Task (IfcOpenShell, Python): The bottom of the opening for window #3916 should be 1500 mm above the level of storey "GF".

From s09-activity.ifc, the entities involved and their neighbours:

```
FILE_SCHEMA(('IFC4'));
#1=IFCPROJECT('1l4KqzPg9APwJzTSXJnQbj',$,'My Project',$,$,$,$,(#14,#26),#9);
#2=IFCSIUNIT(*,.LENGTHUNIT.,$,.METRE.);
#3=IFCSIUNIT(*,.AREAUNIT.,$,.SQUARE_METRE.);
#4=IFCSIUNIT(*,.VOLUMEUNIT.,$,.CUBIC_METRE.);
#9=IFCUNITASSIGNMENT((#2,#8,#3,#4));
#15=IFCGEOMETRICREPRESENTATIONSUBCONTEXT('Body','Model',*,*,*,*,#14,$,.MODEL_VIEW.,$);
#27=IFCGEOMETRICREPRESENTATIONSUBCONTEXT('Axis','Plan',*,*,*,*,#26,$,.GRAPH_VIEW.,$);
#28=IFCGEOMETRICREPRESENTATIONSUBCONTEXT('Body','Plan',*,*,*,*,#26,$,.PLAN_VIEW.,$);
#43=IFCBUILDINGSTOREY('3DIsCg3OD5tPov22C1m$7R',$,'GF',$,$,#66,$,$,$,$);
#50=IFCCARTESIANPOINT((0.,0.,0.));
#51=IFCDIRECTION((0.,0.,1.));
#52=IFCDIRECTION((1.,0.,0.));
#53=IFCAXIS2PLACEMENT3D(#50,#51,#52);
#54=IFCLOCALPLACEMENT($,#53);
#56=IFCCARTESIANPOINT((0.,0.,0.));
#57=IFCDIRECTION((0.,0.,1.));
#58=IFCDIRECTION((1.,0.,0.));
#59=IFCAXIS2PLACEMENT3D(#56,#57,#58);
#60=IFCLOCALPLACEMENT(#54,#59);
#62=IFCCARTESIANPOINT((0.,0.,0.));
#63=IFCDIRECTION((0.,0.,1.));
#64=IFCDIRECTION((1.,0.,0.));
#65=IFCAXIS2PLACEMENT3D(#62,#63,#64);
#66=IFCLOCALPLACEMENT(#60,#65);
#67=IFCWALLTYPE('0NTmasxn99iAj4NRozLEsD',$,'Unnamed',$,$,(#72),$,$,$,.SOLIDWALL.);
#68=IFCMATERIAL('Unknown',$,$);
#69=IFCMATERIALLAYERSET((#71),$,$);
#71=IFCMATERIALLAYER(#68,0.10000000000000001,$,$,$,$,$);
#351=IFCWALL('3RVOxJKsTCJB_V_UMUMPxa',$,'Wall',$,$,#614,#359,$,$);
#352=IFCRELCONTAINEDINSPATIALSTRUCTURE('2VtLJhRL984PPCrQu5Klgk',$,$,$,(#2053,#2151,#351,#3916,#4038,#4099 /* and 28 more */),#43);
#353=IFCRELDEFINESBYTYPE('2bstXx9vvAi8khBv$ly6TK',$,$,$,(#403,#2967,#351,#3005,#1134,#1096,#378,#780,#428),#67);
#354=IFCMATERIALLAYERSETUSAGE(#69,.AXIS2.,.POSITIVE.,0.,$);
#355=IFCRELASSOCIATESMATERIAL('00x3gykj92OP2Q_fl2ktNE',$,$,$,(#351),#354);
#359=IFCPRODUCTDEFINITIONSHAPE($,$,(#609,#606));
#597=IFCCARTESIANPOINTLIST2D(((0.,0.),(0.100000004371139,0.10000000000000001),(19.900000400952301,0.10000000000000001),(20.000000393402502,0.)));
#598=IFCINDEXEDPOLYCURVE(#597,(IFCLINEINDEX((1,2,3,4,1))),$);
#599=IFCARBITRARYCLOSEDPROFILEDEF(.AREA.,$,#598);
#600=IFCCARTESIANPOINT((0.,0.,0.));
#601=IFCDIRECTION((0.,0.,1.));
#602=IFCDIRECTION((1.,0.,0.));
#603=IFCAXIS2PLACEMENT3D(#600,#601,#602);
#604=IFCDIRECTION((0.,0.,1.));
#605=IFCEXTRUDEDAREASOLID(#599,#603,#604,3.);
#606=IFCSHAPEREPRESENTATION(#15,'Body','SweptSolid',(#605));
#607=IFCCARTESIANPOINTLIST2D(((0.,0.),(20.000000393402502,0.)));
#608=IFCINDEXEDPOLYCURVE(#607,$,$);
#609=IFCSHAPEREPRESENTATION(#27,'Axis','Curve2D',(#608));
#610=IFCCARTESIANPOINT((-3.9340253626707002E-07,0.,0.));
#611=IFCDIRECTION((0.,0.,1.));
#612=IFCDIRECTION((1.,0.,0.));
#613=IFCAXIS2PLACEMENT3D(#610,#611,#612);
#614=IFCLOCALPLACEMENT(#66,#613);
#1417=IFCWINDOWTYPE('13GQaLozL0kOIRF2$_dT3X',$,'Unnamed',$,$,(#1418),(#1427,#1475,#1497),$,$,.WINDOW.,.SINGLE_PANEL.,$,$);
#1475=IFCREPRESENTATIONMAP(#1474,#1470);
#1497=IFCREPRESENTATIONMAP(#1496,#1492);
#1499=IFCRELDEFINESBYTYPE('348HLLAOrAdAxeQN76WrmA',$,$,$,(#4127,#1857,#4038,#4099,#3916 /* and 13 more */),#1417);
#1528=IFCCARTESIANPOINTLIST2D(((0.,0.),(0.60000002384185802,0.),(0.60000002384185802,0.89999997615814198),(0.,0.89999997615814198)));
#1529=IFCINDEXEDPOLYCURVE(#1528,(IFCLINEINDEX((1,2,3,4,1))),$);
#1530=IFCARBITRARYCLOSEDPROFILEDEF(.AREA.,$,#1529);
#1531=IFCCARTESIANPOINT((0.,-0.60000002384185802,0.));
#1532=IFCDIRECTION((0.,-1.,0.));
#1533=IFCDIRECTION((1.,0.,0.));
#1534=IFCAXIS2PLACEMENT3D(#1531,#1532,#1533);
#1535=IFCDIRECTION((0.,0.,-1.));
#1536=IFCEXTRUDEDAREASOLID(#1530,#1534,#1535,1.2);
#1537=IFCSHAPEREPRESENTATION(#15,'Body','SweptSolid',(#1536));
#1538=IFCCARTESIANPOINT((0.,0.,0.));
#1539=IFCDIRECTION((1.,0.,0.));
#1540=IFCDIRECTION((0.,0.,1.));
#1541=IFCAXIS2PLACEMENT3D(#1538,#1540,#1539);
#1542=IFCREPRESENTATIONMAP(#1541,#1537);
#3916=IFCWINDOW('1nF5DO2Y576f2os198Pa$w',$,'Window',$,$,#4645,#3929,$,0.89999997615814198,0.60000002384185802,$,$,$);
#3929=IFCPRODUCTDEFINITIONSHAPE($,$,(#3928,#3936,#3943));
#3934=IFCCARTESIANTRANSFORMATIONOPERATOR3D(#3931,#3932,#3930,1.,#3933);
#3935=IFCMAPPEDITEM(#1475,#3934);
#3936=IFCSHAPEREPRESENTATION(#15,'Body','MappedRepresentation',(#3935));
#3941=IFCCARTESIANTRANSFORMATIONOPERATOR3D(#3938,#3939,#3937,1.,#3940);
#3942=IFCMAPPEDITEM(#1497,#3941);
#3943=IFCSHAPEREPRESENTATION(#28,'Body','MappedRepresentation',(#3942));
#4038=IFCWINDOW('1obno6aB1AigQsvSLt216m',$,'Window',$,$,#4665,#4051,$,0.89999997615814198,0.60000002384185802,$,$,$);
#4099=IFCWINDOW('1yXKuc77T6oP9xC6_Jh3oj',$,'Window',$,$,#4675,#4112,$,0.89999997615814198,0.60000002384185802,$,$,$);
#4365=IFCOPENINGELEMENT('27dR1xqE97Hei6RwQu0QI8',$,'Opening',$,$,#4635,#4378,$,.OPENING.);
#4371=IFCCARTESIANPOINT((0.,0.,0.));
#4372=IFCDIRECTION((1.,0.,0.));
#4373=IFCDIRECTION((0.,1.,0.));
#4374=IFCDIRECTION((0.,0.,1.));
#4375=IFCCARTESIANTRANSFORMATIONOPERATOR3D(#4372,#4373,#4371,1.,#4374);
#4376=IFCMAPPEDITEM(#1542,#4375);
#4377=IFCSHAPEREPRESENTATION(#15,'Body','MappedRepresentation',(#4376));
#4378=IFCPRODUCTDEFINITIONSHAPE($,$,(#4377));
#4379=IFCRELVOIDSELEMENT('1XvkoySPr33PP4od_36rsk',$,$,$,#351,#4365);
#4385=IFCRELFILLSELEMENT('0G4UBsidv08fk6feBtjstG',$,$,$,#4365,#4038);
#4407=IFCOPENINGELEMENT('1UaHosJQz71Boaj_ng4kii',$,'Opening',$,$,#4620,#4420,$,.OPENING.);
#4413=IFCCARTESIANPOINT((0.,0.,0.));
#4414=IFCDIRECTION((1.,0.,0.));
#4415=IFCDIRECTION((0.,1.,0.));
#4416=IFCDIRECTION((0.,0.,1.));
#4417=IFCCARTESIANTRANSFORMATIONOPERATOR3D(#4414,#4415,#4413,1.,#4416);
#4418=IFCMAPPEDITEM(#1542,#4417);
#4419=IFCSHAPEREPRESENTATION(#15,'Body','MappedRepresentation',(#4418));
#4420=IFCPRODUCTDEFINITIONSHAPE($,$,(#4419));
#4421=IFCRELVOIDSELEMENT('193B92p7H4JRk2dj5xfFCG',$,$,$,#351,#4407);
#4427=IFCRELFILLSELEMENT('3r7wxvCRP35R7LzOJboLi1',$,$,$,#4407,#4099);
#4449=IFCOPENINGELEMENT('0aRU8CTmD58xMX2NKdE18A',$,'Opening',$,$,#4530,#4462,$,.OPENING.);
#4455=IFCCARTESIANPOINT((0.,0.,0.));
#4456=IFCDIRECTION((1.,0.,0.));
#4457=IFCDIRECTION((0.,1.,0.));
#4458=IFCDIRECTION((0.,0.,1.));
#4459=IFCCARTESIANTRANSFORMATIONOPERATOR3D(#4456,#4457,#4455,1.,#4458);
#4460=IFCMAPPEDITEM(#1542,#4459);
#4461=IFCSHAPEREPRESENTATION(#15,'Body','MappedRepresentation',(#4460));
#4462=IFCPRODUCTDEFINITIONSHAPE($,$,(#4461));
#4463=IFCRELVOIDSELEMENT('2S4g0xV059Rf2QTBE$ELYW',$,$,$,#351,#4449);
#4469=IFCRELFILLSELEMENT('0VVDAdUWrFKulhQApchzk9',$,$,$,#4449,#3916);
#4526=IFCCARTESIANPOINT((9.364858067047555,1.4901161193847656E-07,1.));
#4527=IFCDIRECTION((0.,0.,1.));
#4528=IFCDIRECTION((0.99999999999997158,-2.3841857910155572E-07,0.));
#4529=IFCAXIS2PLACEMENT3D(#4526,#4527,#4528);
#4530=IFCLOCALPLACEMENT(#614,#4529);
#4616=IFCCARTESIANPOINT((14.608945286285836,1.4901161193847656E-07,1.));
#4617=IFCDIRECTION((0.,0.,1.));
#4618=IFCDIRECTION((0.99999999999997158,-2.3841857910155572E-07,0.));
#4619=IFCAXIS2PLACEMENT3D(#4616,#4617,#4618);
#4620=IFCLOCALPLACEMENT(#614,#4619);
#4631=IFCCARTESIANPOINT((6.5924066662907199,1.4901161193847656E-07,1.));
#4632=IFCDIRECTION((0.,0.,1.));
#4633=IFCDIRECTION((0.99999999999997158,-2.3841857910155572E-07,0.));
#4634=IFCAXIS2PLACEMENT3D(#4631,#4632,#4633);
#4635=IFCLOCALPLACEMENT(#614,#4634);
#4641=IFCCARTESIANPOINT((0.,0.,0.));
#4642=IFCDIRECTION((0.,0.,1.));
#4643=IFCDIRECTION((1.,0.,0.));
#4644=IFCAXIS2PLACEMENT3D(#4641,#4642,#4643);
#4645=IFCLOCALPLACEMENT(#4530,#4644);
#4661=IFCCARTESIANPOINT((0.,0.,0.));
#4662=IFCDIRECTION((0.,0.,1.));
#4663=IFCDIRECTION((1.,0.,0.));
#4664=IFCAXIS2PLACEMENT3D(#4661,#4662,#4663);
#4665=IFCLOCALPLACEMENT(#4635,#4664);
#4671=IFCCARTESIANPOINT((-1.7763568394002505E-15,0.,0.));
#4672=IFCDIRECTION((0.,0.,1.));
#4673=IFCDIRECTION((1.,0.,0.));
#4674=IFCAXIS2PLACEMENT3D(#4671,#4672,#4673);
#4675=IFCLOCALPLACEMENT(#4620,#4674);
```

```python
import numpy as np
import ifcopenshell
import ifcopenshell.api.geometry
import ifcopenshell.geom
import ifcopenshell.util.element
import ifcopenshell.util.placement
import ifcopenshell.util.shape
import ifcopenshell.util.unit

model = ifcopenshell.open("s09-activity.ifc")
unit_scale = ifcopenshell.util.unit.calculate_unit_scale(model)

window = model.by_guid("1nF5DO2Y576f2os198Pa$w")
opening = window.FillsVoids[0].RelatingOpeningElement
storey = ifcopenshell.util.element.get_container(window, ifc_class="IfcBuildingStorey")
level = ifcopenshell.util.placement.get_local_placement(storey.ObjectPlacement)[2, 3]

# The opening's origin need not be at the sill, so measure its lowest point.
shape = ifcopenshell.geom.create_shape(ifcopenshell.geom.settings(), opening)
bottom = ifcopenshell.util.shape.get_shape_bottom_elevation(shape, shape.geometry) / unit_scale
dz = level + 1.5 - bottom

shift = np.array([0.0, 0.0, dz])
# The window is placed relative to its opening, so it follows when the opening moves.
matrix = ifcopenshell.util.placement.get_local_placement(opening.ObjectPlacement)
matrix[:3, 3] += shift
ifcopenshell.api.geometry.edit_object_placement(
    model, product=opening, matrix=matrix, is_si=False, should_transform_children=True
)

print(f"moved by {dz * unit_scale:+.3f} m")

model.write("s09-activity-out.ifc")
```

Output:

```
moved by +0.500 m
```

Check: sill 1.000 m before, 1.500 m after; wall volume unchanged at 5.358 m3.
